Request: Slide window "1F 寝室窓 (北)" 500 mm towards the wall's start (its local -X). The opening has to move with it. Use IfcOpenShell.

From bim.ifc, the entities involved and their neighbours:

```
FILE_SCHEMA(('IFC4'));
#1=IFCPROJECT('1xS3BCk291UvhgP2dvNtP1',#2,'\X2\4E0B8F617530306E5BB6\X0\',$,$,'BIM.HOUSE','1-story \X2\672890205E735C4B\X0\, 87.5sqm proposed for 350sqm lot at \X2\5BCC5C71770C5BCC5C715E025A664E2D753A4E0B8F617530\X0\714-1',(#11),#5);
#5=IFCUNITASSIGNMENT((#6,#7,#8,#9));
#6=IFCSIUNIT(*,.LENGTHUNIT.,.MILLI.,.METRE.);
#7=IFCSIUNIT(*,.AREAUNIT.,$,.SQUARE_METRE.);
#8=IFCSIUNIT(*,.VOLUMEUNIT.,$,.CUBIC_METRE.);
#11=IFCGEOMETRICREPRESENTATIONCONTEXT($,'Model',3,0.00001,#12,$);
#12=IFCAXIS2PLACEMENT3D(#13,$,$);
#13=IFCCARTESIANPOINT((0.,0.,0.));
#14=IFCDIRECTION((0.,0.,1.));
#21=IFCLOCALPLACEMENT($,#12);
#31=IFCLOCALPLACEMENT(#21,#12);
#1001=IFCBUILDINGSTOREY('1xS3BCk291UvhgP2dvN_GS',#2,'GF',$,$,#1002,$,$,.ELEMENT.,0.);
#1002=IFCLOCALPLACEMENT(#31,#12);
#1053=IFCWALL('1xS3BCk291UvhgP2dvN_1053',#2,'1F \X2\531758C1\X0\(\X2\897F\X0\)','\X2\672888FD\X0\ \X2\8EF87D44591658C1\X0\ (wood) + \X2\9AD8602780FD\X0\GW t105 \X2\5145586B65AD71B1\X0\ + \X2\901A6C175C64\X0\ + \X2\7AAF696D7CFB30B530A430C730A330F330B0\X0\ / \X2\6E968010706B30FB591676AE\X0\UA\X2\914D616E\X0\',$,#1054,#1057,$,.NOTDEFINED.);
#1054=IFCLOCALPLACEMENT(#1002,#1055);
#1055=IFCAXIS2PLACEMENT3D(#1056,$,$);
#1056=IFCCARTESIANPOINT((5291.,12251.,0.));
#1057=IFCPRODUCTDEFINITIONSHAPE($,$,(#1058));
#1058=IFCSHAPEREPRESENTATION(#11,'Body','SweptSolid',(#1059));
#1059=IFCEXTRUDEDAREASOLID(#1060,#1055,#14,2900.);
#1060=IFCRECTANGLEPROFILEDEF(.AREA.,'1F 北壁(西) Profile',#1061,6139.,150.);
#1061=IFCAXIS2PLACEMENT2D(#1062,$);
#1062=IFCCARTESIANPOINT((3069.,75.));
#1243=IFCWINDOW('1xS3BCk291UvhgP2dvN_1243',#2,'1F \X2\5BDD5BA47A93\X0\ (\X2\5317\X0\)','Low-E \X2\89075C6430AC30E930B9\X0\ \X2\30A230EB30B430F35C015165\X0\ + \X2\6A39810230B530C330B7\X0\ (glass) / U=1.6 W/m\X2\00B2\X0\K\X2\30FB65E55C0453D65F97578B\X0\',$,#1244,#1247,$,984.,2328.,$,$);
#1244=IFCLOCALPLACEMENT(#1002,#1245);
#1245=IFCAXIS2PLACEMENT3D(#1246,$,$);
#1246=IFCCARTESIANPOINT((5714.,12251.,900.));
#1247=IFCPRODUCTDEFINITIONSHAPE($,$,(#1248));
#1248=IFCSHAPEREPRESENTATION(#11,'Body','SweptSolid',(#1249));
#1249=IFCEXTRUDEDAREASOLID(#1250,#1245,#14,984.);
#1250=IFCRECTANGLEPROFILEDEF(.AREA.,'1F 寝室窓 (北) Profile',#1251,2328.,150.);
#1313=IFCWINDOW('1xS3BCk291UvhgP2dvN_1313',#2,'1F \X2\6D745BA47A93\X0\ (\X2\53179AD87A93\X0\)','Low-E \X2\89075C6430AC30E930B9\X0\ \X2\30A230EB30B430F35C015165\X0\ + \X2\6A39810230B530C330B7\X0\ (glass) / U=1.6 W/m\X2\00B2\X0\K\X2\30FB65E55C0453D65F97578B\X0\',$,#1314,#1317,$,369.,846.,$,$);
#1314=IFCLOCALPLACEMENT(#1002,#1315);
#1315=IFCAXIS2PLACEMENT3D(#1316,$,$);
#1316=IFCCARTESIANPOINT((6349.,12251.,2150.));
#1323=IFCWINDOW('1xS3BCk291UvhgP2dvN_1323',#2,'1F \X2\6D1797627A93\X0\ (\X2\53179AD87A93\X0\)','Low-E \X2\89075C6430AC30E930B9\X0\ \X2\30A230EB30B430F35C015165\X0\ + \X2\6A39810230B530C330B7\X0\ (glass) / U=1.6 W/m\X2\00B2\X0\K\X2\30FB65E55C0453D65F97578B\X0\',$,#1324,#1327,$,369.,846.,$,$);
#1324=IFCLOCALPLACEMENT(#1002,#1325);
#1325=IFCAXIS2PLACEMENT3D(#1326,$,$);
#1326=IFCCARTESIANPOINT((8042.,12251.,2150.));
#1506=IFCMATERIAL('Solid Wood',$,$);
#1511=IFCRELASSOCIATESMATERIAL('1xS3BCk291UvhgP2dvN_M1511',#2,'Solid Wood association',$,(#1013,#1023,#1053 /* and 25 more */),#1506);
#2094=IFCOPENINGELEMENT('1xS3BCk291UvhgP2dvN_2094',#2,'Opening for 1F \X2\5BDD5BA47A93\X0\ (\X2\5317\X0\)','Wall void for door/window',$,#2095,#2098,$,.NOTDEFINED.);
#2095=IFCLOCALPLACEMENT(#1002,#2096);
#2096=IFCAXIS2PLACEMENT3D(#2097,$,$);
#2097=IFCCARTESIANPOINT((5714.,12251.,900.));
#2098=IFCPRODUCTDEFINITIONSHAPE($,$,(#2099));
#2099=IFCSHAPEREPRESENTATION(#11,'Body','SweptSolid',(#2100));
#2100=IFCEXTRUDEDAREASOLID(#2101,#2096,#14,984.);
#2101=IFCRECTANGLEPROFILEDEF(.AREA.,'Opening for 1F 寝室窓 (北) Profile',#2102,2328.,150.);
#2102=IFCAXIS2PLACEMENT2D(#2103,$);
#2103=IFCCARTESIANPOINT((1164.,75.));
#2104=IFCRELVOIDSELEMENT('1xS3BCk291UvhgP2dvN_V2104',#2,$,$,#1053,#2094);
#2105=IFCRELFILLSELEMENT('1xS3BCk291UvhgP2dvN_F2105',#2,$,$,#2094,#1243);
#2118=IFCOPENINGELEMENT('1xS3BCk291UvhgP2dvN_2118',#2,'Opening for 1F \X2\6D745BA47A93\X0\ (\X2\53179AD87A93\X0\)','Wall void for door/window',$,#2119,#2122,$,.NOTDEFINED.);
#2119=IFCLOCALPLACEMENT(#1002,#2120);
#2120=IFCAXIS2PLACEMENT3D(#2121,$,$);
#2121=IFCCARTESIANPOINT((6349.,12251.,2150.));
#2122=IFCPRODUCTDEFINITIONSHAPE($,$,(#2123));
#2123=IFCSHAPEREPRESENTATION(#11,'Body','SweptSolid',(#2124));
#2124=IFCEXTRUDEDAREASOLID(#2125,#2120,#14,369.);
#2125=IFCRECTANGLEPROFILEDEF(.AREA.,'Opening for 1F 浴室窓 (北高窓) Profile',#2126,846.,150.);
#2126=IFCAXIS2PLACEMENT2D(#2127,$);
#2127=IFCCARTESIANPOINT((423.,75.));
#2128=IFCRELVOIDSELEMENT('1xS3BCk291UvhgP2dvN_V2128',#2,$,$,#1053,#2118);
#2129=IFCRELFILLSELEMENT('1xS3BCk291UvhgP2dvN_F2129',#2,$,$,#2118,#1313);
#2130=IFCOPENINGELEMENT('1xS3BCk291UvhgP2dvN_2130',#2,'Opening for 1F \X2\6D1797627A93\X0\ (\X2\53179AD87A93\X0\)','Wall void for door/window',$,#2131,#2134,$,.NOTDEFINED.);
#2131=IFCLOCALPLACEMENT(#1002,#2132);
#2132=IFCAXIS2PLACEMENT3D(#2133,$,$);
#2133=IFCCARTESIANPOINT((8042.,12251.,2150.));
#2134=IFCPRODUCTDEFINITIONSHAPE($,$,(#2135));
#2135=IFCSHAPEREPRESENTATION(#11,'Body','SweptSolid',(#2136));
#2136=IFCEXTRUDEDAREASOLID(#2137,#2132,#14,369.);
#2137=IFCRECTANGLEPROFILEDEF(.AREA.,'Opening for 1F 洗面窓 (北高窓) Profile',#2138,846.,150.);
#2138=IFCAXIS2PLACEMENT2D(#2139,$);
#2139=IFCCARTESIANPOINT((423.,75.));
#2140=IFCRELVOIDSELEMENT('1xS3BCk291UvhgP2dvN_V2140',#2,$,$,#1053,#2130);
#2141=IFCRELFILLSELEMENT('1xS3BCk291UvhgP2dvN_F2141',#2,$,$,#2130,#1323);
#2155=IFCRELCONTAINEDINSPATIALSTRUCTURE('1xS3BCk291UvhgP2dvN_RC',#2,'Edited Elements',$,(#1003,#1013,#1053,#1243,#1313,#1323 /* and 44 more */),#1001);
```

```python
import ifcopenshell
import ifcopenshell.api.geometry
import ifcopenshell.util.placement

model = ifcopenshell.open("bim.ifc")

window = model.by_id(1243)
opening = window.FillsVoids[0].RelatingOpeningElement
wall = opening.VoidsElements[0].RelatingBuildingElement

wall_matrix = ifcopenshell.util.placement.get_local_placement(wall.ObjectPlacement)
shift = wall_matrix[:3, 0] * -500.0
before = ifcopenshell.util.placement.get_local_placement(window.ObjectPlacement)[:3, 3].copy()

# The window is not placed relative to its opening, so move both.
for product in (opening, window):
    matrix = ifcopenshell.util.placement.get_local_placement(product.ObjectPlacement)
    matrix[:3, 3] += shift
    ifcopenshell.api.geometry.edit_object_placement(model, product=product, matrix=matrix, is_si=False)

after = ifcopenshell.util.placement.get_local_placement(window.ObjectPlacement)[:3, 3]
print("window moved by", (after - before).round(3) + 0.0)

model.write("bim_rev.ifc")
```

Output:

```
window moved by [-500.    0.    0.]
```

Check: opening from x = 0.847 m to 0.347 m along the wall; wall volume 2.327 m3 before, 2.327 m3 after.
